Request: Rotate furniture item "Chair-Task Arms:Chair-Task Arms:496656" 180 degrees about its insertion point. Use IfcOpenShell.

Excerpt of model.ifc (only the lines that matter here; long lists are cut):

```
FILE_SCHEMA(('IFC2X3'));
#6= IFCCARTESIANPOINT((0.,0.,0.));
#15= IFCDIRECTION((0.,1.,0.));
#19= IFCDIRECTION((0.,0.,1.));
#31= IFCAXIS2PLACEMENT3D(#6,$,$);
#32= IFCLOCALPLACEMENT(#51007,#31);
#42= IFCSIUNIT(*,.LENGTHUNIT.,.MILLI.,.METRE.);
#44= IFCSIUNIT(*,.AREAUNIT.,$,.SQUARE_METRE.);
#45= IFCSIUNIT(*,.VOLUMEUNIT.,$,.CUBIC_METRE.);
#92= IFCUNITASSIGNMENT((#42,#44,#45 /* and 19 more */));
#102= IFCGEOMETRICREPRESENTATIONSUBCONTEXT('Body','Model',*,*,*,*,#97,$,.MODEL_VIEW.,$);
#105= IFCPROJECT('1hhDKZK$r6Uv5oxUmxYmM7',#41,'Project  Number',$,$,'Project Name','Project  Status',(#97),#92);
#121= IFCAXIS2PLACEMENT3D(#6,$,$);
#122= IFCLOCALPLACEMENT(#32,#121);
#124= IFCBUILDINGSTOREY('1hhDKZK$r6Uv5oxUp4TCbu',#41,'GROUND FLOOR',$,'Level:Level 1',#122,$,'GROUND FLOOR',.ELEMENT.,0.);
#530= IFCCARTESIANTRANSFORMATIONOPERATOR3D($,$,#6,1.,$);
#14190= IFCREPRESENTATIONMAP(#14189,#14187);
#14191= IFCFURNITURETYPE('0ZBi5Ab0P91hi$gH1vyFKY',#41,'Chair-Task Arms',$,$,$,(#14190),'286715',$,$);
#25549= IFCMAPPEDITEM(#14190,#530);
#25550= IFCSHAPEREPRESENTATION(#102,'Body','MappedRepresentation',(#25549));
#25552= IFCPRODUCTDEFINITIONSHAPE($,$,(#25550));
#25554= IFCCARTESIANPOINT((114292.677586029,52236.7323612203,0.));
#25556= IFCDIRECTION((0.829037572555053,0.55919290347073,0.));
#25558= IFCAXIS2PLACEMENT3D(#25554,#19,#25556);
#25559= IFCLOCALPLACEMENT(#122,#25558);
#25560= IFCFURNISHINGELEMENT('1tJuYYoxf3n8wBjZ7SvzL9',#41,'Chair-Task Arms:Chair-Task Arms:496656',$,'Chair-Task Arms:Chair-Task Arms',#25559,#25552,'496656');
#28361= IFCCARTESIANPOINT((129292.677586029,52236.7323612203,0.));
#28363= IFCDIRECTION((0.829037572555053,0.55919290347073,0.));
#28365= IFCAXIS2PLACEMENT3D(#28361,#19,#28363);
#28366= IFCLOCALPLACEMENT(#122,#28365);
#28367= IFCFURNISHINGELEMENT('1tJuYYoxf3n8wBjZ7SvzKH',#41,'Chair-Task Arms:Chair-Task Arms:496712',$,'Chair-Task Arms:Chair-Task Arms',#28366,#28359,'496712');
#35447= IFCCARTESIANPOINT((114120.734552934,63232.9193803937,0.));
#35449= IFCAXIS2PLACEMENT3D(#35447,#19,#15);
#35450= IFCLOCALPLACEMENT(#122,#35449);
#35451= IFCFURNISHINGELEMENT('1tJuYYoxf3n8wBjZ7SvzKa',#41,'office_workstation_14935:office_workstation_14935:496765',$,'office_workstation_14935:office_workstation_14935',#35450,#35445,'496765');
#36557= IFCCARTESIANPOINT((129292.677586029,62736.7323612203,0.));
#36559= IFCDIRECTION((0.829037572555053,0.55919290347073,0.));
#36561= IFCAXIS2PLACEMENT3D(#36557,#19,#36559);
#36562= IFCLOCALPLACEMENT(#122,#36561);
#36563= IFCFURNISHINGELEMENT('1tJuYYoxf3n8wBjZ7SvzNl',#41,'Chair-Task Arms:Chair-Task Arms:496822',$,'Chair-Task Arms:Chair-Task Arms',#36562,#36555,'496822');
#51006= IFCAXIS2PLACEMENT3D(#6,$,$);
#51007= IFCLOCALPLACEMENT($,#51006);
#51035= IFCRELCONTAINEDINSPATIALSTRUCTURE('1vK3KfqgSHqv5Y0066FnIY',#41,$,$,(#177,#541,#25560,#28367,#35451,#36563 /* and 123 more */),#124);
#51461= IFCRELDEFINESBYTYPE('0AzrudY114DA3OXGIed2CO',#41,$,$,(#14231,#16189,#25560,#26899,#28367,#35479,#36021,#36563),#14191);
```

```python
import ifcopenshell
import ifcopenshell.api.geometry
import ifcopenshell.util.placement

model = ifcopenshell.open("model.ifc")

item = model.by_guid("1tJuYYoxf3n8wBjZ7SvzL9")
matrix = ifcopenshell.util.placement.get_local_placement(item.ObjectPlacement)
matrix = matrix @ ifcopenshell.util.placement.rotation(180, "Z")
ifcopenshell.api.geometry.edit_object_placement(model, product=item, matrix=matrix, is_si=False)

print(ifcopenshell.util.placement.get_local_placement(item.ObjectPlacement).round(3) + 0.0)

model.write("model_v2.ifc")
```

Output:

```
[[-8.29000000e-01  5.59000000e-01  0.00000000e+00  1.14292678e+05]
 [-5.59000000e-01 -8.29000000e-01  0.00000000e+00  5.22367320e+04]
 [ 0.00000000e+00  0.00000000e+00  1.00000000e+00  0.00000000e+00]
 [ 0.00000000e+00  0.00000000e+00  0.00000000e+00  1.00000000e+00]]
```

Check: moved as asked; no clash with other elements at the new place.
